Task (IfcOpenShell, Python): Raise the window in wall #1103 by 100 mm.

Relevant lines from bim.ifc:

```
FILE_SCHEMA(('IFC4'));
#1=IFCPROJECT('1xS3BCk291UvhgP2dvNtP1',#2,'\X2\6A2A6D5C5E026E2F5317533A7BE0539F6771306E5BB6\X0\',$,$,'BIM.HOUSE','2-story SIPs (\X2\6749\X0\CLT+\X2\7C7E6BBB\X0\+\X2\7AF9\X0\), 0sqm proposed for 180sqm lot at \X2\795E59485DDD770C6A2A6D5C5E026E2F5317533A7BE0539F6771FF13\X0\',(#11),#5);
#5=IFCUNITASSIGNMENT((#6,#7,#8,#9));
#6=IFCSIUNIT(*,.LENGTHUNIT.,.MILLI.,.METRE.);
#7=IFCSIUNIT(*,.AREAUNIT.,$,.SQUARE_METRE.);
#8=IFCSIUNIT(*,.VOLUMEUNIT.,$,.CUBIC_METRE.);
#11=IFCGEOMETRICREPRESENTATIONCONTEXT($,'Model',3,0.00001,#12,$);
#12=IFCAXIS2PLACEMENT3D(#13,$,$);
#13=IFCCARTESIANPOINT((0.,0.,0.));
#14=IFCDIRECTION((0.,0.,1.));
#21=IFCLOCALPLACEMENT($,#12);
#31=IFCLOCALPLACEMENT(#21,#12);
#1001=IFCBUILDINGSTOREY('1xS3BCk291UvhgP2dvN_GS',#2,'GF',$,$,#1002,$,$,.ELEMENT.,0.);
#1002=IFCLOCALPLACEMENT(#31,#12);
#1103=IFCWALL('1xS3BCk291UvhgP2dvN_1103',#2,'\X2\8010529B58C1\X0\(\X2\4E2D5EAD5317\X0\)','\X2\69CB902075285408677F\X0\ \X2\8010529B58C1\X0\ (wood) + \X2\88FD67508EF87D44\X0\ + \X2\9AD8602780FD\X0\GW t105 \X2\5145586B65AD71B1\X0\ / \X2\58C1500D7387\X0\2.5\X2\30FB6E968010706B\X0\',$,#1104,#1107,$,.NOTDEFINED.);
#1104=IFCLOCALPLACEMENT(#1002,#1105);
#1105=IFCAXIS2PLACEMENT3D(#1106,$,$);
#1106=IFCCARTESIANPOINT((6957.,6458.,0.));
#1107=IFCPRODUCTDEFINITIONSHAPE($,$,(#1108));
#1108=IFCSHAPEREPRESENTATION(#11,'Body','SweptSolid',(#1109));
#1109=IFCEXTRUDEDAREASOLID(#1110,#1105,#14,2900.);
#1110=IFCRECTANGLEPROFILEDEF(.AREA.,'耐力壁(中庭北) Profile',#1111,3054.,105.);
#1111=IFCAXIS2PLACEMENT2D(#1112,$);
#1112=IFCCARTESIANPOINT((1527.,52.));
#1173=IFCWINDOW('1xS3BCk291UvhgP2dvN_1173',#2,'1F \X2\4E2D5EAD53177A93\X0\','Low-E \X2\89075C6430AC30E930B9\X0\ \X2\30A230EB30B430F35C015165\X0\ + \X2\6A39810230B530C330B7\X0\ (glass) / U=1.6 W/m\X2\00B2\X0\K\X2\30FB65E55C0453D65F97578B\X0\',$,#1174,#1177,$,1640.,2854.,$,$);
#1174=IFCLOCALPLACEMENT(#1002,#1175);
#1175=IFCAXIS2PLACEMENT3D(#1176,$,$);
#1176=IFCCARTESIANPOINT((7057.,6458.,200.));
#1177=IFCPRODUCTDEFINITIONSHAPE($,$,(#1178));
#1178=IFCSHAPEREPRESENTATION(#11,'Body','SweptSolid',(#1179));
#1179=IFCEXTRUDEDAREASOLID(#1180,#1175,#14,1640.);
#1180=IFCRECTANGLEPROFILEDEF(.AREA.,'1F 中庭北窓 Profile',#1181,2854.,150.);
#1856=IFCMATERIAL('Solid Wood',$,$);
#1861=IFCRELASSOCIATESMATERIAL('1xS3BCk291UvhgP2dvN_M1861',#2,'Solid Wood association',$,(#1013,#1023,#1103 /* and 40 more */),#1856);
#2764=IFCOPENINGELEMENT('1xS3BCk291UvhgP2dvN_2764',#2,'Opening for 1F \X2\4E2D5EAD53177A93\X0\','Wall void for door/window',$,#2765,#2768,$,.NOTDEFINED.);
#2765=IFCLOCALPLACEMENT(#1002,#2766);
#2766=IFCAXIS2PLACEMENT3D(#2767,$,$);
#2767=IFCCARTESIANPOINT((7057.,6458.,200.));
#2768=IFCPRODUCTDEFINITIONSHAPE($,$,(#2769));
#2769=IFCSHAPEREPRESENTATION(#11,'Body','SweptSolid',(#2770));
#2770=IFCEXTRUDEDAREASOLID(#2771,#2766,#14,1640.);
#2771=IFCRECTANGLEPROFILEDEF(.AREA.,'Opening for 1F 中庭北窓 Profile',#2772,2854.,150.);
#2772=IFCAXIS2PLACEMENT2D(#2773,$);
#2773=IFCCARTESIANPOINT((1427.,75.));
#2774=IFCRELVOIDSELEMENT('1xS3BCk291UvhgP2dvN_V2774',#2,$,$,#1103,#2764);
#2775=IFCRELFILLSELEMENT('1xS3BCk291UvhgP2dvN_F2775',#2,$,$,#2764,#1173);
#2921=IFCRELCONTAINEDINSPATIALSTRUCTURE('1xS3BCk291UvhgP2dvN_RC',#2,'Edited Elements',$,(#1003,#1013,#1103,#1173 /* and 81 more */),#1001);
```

```python
import numpy as np
import ifcopenshell
import ifcopenshell.api.geometry
import ifcopenshell.util.placement
import ifcopenshell.util.unit

model = ifcopenshell.open("bim.ifc")
unit_scale = ifcopenshell.util.unit.calculate_unit_scale(model)

window = model.by_guid("1xS3BCk291UvhgP2dvN_1173")
opening = window.FillsVoids[0].RelatingOpeningElement
dz = 0.1 / unit_scale

shift = np.array([0.0, 0.0, dz])
# The window is not placed relative to its opening, so move both.
for product in (opening, window):
    matrix = ifcopenshell.util.placement.get_local_placement(product.ObjectPlacement)
    matrix[:3, 3] += shift
    ifcopenshell.api.geometry.edit_object_placement(model, product=product, matrix=matrix, is_si=False)

print(f"moved by {dz * unit_scale:+.3f} m")

model.write("bim_v2.ifc")
```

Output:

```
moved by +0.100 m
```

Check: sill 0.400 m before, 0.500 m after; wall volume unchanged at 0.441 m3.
